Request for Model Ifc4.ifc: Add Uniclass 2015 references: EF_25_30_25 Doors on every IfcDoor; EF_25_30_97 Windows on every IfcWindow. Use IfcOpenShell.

First a look at what the model holds.

```python
import ifcopenshell

model = ifcopenshell.open("Model Ifc4.ifc")
print(model.schema)
print("classifications:", [c.Name for c in model.by_type("IfcClassification")])
for ifc_class in ("IfcDoor", "IfcRoof", "IfcStair", "IfcWall", "IfcWindow"):
    print(ifc_class, len(model.by_type(ifc_class)))
```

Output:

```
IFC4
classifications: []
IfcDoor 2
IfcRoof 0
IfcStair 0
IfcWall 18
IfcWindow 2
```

```python
import ifcopenshell
import ifcopenshell.api.classification

model = ifcopenshell.open("Model Ifc4.ifc")

system = ifcopenshell.api.classification.add_classification(model, classification="Uniclass 2015")

codes = {
    "IfcDoor": ("EF_25_30_25", "Doors"),
    "IfcWindow": ("EF_25_30_97", "Windows"),
}
for ifc_class, (code, name) in codes.items():
    products = model.by_type(ifc_class)
    ifcopenshell.api.classification.add_reference(
        model, products=products, classification=system, identification=code, name=name
    )
    print(code, len(products))

model.write("Model Ifc4_updated.ifc")
```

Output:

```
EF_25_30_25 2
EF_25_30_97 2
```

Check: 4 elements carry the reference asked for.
